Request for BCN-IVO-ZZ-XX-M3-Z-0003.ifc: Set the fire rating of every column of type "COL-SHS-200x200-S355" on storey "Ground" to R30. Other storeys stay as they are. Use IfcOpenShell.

First a look at what the model holds.

```python
import ifcopenshell
import ifcopenshell.util.element

model = ifcopenshell.open("BCN-IVO-ZZ-XX-M3-Z-0003.ifc")
print(model.schema)
storey = next(s for s in model.by_type("IfcBuildingStorey") if s.Name == "Ground")
columns = [e for e in ifcopenshell.util.element.get_decomposition(storey) if e.is_a("IfcColumn")]
seen = {}
for e in columns:
    element_type = ifcopenshell.util.element.get_type(e)
    key = (element_type.Name if element_type != e and element_type else None, ifcopenshell.util.element.get_pset(e, "Pset_ColumnCommon", "FireRating"))
    seen[key] = seen.get(key, 0) + 1
for (name, value), count in sorted(seen.items(), key=str):
    print(count, "x", name, "|", value)
```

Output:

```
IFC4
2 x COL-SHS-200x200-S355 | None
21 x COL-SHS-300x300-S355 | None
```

```python
import ifcopenshell
import ifcopenshell.api.pset
import ifcopenshell.util.element

model = ifcopenshell.open("BCN-IVO-ZZ-XX-M3-Z-0003.ifc")

storey = next(s for s in model.by_type("IfcBuildingStorey") if s.Name == "Ground")
columns = [e for e in ifcopenshell.util.element.get_decomposition(storey) if e.is_a("IfcColumn")]

count = 0
for e in columns:
    element_type = ifcopenshell.util.element.get_type(e)
    if element_type in (None, e) or element_type.Name != "COL-SHS-200x200-S355":
        continue
    # add_pset returns the element's existing set when there is one.
    pset = ifcopenshell.api.pset.add_pset(model, product=e, name="Pset_ColumnCommon")
    ifcopenshell.api.pset.edit_pset(model, pset=pset, properties={"FireRating": "R30"})
    count += 1

print(count, "columns updated")

model.write("BCN-IVO-ZZ-XX-M3-Z-0003_rev.ifc")
```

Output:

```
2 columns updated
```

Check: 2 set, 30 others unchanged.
